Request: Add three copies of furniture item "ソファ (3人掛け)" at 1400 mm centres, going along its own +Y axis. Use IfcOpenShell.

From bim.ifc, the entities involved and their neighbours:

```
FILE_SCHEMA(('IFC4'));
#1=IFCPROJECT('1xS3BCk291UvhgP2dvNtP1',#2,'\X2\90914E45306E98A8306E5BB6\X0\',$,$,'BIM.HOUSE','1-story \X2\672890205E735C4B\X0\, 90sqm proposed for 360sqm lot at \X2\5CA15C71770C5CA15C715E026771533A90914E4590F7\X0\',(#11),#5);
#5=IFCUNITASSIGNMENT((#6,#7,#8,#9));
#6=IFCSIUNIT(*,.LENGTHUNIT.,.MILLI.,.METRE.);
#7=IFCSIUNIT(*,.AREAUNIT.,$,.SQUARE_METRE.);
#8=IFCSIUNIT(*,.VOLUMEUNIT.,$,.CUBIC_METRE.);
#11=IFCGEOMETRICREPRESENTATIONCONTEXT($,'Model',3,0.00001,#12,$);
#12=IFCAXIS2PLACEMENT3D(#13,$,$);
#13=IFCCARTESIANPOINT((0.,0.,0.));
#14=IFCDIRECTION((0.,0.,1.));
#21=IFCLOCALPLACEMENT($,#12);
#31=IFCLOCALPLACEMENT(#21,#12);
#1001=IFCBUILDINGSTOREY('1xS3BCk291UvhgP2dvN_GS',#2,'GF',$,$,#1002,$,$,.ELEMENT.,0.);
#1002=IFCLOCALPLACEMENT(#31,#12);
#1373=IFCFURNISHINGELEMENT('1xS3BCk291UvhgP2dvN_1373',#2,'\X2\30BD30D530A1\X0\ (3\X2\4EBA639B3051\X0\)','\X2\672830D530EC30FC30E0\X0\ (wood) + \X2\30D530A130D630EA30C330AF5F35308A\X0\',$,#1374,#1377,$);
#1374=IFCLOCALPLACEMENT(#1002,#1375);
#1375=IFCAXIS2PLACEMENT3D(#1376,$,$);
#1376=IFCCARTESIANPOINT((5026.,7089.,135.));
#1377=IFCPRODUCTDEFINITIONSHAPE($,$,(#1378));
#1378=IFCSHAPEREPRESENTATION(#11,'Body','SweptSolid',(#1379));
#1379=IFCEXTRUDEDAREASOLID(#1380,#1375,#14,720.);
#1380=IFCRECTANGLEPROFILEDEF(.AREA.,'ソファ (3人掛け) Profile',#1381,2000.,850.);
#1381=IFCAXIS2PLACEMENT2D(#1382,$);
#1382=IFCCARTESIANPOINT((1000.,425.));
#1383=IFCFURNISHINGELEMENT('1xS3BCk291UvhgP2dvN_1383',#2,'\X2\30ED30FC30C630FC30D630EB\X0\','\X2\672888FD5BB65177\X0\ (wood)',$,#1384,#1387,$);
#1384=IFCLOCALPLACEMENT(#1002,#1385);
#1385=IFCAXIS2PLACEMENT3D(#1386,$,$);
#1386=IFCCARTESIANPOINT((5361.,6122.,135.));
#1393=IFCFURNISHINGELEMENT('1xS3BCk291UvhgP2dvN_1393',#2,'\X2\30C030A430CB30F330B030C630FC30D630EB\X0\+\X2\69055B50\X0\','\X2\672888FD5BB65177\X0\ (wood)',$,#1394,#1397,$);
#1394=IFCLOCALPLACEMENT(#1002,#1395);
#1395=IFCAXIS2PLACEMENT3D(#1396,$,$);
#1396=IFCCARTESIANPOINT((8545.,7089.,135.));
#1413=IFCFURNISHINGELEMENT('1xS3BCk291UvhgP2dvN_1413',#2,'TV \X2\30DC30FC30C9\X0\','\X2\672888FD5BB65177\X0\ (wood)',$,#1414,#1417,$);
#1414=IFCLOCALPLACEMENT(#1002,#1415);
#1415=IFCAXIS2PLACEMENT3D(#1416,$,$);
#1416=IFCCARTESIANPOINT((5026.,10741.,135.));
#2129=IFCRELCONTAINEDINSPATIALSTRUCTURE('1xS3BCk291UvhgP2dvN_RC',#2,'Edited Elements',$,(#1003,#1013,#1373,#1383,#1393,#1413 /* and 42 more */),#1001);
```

```python
import ifcopenshell
import ifcopenshell.api.geometry
import ifcopenshell.api.root
import ifcopenshell.util.element
import ifcopenshell.util.placement
import ifcopenshell.util.unit

model = ifcopenshell.open("bim.ifc")
unit_scale = ifcopenshell.util.unit.calculate_unit_scale(model)


def reuse_history(source, copy):
    """copy_class also copies each property set's owner history, people and application; keep the originals."""
    for rel in copy.IsDefinedBy:
        if rel.is_a("IfcRelDefinesByProperties") and (history := rel.RelatingPropertyDefinition.OwnerHistory):
            rel.RelatingPropertyDefinition.OwnerHistory = source.OwnerHistory
            ifcopenshell.util.element.remove_deep2(model, history)


source = model.by_guid("1xS3BCk291UvhgP2dvN_1373")
base = ifcopenshell.util.placement.get_local_placement(source.ObjectPlacement)
step = base[:3, 1] * 1.4 / unit_scale

for i in range(1, 4):
    copy = ifcopenshell.api.root.copy_class(model, product=source)
    copy.Representation = ifcopenshell.util.element.copy_deep(
        model, source.Representation, exclude=["IfcGeometricRepresentationContext", "IfcRepresentationMap"]
    )
    reuse_history(source, copy)
    matrix = base.copy()
    matrix[:3, 3] += i * step
    print("added at", matrix[:3, 3].round(3) + 0.0)
    ifcopenshell.api.geometry.edit_object_placement(model, product=copy, matrix=matrix, is_si=False)

model.write("bim_edited.ifc")
```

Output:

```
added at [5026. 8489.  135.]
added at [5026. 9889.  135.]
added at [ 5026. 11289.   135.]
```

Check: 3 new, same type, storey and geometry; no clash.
